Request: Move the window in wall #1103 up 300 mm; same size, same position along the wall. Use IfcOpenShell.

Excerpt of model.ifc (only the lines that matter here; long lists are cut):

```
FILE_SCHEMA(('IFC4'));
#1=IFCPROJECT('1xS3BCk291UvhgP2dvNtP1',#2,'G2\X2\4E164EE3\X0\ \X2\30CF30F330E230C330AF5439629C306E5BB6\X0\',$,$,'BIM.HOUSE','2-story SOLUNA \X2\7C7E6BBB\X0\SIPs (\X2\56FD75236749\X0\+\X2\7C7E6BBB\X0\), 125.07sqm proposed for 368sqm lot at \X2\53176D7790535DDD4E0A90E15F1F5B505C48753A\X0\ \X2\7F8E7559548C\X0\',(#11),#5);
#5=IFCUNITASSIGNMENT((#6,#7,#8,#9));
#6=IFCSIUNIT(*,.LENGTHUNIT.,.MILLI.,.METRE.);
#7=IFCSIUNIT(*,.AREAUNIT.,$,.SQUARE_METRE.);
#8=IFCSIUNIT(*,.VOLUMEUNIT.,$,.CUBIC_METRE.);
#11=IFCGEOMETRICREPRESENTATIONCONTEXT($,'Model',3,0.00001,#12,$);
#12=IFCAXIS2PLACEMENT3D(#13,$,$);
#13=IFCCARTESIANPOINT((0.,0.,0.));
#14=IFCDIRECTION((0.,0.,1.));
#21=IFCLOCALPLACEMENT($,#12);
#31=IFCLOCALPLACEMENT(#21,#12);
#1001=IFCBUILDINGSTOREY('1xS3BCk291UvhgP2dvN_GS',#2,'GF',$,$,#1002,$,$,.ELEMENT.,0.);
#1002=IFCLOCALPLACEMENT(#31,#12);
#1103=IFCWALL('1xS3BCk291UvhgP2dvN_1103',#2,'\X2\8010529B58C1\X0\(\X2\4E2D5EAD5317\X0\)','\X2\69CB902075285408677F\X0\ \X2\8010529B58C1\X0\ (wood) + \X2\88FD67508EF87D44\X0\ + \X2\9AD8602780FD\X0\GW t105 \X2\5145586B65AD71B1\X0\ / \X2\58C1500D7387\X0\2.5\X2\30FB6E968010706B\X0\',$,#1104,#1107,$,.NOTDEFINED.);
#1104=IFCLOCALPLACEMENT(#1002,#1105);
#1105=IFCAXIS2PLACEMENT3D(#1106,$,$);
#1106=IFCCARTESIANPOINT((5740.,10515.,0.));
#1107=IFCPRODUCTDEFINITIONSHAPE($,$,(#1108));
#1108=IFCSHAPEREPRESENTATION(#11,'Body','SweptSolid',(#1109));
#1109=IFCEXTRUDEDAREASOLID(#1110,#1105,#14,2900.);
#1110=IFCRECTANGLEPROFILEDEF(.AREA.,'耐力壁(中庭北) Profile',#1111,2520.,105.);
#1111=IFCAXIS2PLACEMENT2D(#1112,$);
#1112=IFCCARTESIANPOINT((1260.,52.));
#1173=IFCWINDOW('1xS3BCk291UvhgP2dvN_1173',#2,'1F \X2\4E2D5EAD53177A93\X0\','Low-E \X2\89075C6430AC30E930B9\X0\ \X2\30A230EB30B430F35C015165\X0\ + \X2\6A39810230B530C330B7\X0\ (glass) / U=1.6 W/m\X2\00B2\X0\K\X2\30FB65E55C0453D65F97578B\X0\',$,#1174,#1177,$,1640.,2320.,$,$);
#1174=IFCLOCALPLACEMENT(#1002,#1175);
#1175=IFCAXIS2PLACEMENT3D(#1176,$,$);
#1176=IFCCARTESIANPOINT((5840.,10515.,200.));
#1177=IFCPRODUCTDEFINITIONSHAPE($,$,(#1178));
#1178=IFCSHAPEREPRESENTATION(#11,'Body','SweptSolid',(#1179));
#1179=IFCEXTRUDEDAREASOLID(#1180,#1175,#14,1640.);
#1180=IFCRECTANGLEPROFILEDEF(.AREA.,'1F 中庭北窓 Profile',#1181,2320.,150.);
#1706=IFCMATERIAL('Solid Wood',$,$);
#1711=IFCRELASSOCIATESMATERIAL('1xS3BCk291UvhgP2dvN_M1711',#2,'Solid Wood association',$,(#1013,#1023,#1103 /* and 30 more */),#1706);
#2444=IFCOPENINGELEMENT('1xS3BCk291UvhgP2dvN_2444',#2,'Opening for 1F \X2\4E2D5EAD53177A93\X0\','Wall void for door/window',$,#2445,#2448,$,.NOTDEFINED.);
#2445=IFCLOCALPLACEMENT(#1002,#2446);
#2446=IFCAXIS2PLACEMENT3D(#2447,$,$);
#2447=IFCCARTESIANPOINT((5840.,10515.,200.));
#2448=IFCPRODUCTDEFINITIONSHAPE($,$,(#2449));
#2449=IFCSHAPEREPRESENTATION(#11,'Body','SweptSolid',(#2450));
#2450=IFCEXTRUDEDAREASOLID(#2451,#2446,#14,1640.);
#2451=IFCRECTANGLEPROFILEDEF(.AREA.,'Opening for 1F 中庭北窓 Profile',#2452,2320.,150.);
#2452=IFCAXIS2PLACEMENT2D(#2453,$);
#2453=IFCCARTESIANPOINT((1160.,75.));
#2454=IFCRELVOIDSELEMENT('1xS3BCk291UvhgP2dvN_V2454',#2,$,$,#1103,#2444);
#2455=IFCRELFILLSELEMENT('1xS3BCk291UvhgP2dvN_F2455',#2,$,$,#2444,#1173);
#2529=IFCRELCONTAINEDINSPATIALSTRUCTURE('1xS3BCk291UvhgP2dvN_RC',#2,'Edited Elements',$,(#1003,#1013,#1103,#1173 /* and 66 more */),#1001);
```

```python
import numpy as np
import ifcopenshell
import ifcopenshell.api.geometry
import ifcopenshell.util.placement
import ifcopenshell.util.unit

model = ifcopenshell.open("model.ifc")
unit_scale = ifcopenshell.util.unit.calculate_unit_scale(model)

window = model.by_guid("1xS3BCk291UvhgP2dvN_1173")
opening = window.FillsVoids[0].RelatingOpeningElement
dz = 300.0

shift = np.array([0.0, 0.0, dz])
# The window is not placed relative to its opening, so move both.
for product in (opening, window):
    matrix = ifcopenshell.util.placement.get_local_placement(product.ObjectPlacement)
    matrix[:3, 3] += shift
    ifcopenshell.api.geometry.edit_object_placement(model, product=product, matrix=matrix, is_si=False)

print(f"moved by {dz * unit_scale:+.3f} m")

model.write("model-out.ifc")
```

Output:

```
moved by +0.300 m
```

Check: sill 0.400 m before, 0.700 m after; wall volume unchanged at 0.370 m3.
